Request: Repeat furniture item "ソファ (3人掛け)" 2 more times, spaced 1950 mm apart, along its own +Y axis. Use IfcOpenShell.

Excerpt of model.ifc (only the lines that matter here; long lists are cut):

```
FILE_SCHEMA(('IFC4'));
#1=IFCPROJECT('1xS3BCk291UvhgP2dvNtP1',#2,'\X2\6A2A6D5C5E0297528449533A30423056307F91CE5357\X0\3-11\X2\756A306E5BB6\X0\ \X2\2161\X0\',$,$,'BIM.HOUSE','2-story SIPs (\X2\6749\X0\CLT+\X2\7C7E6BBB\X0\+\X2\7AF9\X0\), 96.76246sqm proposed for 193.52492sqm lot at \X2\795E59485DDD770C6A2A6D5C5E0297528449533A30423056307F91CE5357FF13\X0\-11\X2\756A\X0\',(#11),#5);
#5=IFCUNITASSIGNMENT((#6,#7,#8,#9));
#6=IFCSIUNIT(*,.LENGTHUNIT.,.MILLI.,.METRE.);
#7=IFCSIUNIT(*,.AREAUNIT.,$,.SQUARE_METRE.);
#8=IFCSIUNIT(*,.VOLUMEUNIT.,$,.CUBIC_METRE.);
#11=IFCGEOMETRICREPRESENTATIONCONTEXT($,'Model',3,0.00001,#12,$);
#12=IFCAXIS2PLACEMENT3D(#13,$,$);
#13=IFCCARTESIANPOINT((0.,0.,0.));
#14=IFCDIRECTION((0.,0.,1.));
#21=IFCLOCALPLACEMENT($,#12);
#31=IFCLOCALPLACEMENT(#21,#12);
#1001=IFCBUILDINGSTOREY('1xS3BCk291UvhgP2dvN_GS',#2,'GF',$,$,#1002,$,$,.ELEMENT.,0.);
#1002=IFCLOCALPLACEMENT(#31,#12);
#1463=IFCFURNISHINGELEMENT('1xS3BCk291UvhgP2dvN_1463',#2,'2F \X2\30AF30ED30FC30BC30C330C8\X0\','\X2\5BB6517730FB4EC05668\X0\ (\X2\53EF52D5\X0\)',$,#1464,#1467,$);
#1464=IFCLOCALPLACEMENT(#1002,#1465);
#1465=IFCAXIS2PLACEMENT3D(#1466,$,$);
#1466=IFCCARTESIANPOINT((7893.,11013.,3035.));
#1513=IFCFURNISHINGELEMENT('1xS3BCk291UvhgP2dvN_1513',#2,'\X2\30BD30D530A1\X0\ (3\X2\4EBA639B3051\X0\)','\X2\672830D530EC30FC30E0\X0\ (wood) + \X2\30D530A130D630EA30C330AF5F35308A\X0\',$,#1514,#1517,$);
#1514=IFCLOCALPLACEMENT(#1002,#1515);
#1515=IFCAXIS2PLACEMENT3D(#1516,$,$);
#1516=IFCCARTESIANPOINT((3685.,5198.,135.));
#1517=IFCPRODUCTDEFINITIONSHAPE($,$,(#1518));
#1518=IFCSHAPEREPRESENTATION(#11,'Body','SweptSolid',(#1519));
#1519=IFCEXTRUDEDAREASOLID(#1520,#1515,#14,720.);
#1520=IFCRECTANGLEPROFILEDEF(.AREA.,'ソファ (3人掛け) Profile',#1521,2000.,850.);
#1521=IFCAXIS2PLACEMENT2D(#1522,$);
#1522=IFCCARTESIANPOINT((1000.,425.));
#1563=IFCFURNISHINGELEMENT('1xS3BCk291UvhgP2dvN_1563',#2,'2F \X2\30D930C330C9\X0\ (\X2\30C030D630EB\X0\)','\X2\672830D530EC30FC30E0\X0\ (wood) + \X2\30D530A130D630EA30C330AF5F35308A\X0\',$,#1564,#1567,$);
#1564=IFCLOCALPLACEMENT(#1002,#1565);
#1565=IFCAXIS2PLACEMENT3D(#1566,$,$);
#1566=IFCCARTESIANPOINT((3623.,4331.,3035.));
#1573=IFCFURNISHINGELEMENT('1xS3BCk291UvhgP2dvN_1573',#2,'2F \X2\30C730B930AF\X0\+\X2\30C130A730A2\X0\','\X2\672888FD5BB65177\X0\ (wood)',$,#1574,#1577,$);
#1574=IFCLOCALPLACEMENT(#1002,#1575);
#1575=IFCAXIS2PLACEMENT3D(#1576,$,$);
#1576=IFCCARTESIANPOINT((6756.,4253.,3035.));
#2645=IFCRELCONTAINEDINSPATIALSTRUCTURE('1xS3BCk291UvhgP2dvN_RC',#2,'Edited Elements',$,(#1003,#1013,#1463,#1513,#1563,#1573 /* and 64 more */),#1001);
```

```python
import ifcopenshell
import ifcopenshell.api.geometry
import ifcopenshell.api.root
import ifcopenshell.util.element
import ifcopenshell.util.placement

model = ifcopenshell.open("model.ifc")


def reuse_history(source, copy):
    """copy_class also copies each property set's owner history, people and application; keep the originals."""
    for rel in copy.IsDefinedBy:
        if rel.is_a("IfcRelDefinesByProperties") and (history := rel.RelatingPropertyDefinition.OwnerHistory):
            rel.RelatingPropertyDefinition.OwnerHistory = source.OwnerHistory
            ifcopenshell.util.element.remove_deep2(model, history)


source = model.by_id(1513)
base = ifcopenshell.util.placement.get_local_placement(source.ObjectPlacement)
step = base[:3, 1] * 1950.0

for i in range(1, 3):
    copy = ifcopenshell.api.root.copy_class(model, product=source)
    copy.Representation = ifcopenshell.util.element.copy_deep(
        model, source.Representation, exclude=["IfcGeometricRepresentationContext", "IfcRepresentationMap"]
    )
    reuse_history(source, copy)
    matrix = base.copy()
    matrix[:3, 3] += i * step
    print("added at", matrix[:3, 3].round(3) + 0.0)
    ifcopenshell.api.geometry.edit_object_placement(model, product=copy, matrix=matrix, is_si=False)

model.write("model_rev.ifc")
```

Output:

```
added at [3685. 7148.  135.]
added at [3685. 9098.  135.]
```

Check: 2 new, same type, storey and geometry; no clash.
